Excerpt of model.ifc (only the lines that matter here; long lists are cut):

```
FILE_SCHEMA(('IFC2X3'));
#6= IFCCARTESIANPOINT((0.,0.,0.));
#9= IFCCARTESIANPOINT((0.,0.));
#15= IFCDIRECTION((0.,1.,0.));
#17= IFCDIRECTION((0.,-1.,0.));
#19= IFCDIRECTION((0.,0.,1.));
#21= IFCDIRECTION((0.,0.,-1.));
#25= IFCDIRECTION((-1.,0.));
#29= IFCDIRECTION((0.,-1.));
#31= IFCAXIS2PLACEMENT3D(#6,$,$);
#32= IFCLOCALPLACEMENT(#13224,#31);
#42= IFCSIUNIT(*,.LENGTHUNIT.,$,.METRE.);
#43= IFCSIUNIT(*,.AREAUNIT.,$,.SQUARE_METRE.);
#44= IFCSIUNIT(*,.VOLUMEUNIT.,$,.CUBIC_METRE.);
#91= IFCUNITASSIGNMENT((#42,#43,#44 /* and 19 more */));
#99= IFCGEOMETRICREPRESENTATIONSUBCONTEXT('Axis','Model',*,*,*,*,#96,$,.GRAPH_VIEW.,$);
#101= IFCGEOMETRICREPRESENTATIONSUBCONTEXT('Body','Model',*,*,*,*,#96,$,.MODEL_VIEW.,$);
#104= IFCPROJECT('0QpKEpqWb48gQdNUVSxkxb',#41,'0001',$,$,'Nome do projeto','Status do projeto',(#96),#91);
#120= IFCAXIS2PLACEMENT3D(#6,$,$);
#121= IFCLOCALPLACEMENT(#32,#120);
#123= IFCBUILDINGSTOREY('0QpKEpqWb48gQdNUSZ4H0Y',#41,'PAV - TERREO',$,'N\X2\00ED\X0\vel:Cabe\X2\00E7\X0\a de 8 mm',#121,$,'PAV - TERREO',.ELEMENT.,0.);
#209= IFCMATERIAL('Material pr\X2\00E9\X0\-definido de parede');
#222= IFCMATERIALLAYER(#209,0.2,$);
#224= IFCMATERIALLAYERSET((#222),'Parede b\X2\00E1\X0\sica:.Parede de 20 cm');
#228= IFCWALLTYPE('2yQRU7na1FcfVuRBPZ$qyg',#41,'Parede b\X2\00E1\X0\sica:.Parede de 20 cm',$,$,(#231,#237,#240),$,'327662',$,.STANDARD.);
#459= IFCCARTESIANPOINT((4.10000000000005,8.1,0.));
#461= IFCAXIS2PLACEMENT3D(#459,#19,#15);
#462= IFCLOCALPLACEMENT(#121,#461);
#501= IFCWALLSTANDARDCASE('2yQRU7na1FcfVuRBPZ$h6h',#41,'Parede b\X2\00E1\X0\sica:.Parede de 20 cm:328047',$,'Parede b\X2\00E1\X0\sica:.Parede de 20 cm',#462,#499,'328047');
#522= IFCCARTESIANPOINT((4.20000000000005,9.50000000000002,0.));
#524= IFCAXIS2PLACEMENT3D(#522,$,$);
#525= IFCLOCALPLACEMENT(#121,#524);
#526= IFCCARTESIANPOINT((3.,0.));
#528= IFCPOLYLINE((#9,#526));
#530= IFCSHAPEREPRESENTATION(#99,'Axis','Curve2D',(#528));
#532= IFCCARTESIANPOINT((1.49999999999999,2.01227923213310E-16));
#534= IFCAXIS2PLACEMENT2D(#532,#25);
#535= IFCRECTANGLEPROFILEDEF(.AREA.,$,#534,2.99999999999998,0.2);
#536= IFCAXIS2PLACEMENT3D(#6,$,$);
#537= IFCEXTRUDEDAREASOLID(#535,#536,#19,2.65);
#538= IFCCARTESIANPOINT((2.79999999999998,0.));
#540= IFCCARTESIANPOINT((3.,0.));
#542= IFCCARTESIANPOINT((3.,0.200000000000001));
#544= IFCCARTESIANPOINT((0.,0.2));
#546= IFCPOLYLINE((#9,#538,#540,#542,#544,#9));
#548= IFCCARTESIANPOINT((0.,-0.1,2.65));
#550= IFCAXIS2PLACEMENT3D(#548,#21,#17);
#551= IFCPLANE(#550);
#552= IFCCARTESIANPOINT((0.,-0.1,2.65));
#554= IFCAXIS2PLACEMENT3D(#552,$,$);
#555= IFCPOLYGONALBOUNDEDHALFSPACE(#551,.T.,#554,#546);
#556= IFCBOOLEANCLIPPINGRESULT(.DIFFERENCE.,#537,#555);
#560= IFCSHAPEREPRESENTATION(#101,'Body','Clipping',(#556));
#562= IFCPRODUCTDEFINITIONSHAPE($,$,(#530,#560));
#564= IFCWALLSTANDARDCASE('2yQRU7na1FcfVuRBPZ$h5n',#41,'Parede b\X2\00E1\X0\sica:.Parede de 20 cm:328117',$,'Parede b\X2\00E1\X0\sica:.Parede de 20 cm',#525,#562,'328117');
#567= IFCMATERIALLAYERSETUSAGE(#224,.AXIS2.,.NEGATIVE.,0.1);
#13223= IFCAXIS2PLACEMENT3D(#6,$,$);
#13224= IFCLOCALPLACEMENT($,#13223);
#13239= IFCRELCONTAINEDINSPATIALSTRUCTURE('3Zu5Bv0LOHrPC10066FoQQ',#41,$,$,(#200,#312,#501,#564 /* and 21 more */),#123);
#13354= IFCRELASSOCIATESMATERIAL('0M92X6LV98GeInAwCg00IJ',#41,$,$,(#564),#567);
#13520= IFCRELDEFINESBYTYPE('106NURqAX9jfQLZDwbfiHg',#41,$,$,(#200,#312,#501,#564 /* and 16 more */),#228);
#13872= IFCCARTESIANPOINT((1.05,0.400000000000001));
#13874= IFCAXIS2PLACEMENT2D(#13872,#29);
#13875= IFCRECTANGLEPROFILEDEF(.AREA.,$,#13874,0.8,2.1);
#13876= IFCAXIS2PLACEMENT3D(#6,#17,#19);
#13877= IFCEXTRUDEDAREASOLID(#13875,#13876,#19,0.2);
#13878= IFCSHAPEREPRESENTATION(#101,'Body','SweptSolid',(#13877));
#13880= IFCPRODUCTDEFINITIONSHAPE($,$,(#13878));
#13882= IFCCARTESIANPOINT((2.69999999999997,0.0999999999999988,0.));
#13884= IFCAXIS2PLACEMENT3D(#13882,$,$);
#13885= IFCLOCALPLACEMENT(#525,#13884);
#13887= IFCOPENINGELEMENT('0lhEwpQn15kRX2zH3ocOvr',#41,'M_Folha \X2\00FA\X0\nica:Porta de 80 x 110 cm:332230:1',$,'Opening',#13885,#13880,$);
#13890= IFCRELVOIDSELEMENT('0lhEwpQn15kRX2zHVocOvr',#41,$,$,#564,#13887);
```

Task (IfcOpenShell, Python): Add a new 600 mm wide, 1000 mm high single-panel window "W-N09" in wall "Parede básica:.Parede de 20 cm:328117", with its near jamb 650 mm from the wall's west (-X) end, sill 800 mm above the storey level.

```python
import numpy as np
import ifcopenshell
import ifcopenshell.api.feature
import ifcopenshell.api.geometry
import ifcopenshell.api.root
import ifcopenshell.api.spatial
import ifcopenshell.api.type
import ifcopenshell.geom
import ifcopenshell.util.element
import ifcopenshell.util.placement
import ifcopenshell.util.representation
import ifcopenshell.util.shape
import ifcopenshell.util.unit

model = ifcopenshell.open("model.ifc")
unit_scale = ifcopenshell.util.unit.calculate_unit_scale(model)
settings = ifcopenshell.geom.settings()


def volume(element):
    """Net volume in cubic metres, openings subtracted."""
    shape = ifcopenshell.geom.create_shape(settings, element)
    return ifcopenshell.util.shape.get_volume(shape.geometry)


wall = model.by_id(564)
storey = ifcopenshell.util.element.get_container(wall, ifc_class="IfcBuildingStorey")
context = ifcopenshell.util.representation.get_context(model, "Model", "Body", "MODEL_VIEW")
before = volume(wall)

width, height, from_end, sill = 0.6, 1, 0.65, 0.8  # metres

# The wall runs along its own X axis, and the end named is its -X end.
wall_shape = ifcopenshell.geom.create_shape(settings, wall)
x, y, z = ifcopenshell.util.shape.get_vertices(wall_shape.geometry).T
start = x.min() + from_end
face, thickness = float(y.min()), float(y.max() - y.min())
wall_matrix = ifcopenshell.util.placement.get_local_placement(wall.ObjectPlacement)
level = ifcopenshell.util.placement.get_local_placement(storey.ObjectPlacement)[2, 3]


def in_wall(x, y):
    """Placement at x, y metres in the wall's axes, at sill height."""
    matrix = wall_matrix.copy()
    matrix[:, 3] = wall_matrix @ np.array([x / unit_scale, y / unit_scale, 0.0, 1.0])
    matrix[2, 3] = level + sill / unit_scale
    return matrix


# Opening: a box that overshoots both wall faces by 50 mm.
opening = ifcopenshell.api.root.create_entity(model, ifc_class="IfcOpeningElement")
box = ifcopenshell.api.geometry.add_wall_representation(
    model, context=context, length=width, height=height, thickness=thickness + 0.1
)
ifcopenshell.api.geometry.assign_representation(model, product=opening, representation=box)
ifcopenshell.api.geometry.edit_object_placement(model, product=opening, matrix=in_wall(start, face - 0.05), is_si=False)
ifcopenshell.api.feature.add_feature(model, feature=opening, element=wall)

window = ifcopenshell.api.root.create_entity(model, ifc_class="IfcWindow", name="W-N09")
window.OverallWidth, window.OverallHeight = width / unit_scale, height / unit_scale
body = ifcopenshell.api.geometry.add_window_representation(
    model,
    context=context,
    overall_width=window.OverallWidth,
    overall_height=window.OverallHeight,
    partition_type="SINGLE_PANEL",
)
ifcopenshell.api.geometry.assign_representation(model, product=window, representation=body)
ifcopenshell.api.spatial.assign_container(model, products=[window], relating_structure=storey)
fills = ifcopenshell.api.feature.add_filling(model, opening=opening, element=window)
fills.OwnerHistory = window.OwnerHistory  # required in IFC2X3

# IFC2X3 keeps the operation on the window style.
style = ifcopenshell.api.root.create_entity(model, ifc_class="IfcWindowStyle", name="W-N09")
style.OperationType, style.ConstructionType = "SINGLE_PANEL", "NOTDEFINED"
style.ParameterTakesPrecedence = style.Sizeable = False
ifcopenshell.api.type.assign_type(model, related_objects=[window], relating_type=style)

# Centre the window in the wall's thickness.
ifcopenshell.api.geometry.edit_object_placement(model, product=window, matrix=in_wall(start, face), is_si=False)
window_shape = ifcopenshell.geom.create_shape(settings, window)
depth = ifcopenshell.util.shape.get_vertices(window_shape.geometry)[:, 1]
offset = face + thickness / 2 - (depth.min() + depth.max()) / 2
ifcopenshell.api.geometry.edit_object_placement(model, product=window, matrix=in_wall(start, offset), is_si=False)

after = volume(wall)

print(f"wall volume {before:.3f} -> {after:.3f} m3")

model.write("model_rev.ifc")
```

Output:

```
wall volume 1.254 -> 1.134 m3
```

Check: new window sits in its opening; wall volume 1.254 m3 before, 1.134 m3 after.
